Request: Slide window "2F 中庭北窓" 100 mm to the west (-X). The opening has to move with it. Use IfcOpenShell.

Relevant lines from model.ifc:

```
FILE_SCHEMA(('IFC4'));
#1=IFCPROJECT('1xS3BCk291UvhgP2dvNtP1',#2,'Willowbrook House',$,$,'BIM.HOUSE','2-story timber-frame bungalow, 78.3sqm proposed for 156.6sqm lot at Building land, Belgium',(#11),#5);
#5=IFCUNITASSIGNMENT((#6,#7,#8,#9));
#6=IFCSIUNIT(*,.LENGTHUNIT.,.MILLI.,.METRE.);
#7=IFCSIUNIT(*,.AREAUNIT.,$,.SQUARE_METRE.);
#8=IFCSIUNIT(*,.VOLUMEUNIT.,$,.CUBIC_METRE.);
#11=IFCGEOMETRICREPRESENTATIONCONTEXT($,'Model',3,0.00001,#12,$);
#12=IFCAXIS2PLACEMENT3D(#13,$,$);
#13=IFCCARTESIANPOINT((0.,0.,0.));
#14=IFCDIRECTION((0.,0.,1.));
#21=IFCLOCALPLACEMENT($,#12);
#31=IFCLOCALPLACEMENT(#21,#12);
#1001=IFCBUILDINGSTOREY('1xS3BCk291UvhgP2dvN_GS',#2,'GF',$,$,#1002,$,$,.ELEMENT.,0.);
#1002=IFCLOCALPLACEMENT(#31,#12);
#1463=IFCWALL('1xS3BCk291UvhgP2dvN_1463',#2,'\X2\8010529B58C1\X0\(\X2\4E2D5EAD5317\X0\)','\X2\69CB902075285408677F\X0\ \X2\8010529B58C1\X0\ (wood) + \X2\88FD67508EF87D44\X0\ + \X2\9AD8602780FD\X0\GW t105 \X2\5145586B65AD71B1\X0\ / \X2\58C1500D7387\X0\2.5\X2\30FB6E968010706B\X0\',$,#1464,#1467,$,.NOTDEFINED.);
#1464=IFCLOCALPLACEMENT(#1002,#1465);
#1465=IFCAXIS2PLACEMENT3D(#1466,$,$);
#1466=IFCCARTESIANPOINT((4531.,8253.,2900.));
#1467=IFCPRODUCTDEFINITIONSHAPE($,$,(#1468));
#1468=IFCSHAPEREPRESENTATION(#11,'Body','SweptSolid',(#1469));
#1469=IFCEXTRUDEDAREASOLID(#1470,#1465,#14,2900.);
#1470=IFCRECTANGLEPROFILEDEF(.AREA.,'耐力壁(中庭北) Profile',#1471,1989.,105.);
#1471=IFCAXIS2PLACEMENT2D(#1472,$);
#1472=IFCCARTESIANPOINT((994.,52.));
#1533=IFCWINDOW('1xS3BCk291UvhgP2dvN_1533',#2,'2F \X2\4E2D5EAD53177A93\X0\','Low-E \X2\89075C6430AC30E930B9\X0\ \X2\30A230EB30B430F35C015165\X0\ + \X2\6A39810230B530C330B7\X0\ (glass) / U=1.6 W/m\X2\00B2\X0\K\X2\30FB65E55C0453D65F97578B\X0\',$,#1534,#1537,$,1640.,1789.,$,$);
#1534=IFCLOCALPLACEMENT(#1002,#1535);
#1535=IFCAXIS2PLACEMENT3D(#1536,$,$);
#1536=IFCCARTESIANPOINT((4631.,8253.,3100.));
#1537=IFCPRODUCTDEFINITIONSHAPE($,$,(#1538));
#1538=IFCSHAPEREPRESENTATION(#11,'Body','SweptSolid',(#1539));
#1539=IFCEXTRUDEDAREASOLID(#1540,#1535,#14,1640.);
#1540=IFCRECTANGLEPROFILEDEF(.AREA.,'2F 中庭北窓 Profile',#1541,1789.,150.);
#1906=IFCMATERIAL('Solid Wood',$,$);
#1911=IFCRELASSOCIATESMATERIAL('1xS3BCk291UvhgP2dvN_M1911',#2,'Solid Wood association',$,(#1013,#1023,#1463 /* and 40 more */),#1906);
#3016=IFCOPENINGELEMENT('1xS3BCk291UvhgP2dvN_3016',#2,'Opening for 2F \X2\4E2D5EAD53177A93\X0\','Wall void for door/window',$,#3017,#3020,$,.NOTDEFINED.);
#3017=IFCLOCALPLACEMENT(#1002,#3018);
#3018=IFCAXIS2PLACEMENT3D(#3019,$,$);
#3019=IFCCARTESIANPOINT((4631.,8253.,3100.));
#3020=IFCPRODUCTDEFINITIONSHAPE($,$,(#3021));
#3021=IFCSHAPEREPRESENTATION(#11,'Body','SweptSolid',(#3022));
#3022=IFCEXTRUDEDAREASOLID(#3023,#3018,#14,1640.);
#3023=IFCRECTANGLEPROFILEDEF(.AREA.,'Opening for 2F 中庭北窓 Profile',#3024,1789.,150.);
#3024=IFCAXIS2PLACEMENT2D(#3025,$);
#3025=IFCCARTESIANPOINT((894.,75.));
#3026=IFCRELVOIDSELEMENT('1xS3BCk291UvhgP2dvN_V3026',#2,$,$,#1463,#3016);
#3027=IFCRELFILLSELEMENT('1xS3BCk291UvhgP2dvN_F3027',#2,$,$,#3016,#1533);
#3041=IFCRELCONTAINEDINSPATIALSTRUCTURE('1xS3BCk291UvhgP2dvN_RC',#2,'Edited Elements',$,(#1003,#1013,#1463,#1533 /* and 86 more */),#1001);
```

```python
import ifcopenshell
import ifcopenshell.api.geometry
import ifcopenshell.util.placement
import ifcopenshell.util.unit

model = ifcopenshell.open("model.ifc")
unit_scale = ifcopenshell.util.unit.calculate_unit_scale(model)

window = model.by_id(1533)
opening = window.FillsVoids[0].RelatingOpeningElement
wall = opening.VoidsElements[0].RelatingBuildingElement

wall_matrix = ifcopenshell.util.placement.get_local_placement(wall.ObjectPlacement)
shift = wall_matrix[:3, 0] * -0.1 / unit_scale
before = ifcopenshell.util.placement.get_local_placement(window.ObjectPlacement)[:3, 3].copy()

# The window is not placed relative to its opening, so move both.
for product in (opening, window):
    matrix = ifcopenshell.util.placement.get_local_placement(product.ObjectPlacement)
    matrix[:3, 3] += shift
    ifcopenshell.api.geometry.edit_object_placement(model, product=product, matrix=matrix, is_si=False)

after = ifcopenshell.util.placement.get_local_placement(window.ObjectPlacement)[:3, 3]
print("window moved by", (after - before).round(3) + 0.0)

model.write("model_updated.ifc")
```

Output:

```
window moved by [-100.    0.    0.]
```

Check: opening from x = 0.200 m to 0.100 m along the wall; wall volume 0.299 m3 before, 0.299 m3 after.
